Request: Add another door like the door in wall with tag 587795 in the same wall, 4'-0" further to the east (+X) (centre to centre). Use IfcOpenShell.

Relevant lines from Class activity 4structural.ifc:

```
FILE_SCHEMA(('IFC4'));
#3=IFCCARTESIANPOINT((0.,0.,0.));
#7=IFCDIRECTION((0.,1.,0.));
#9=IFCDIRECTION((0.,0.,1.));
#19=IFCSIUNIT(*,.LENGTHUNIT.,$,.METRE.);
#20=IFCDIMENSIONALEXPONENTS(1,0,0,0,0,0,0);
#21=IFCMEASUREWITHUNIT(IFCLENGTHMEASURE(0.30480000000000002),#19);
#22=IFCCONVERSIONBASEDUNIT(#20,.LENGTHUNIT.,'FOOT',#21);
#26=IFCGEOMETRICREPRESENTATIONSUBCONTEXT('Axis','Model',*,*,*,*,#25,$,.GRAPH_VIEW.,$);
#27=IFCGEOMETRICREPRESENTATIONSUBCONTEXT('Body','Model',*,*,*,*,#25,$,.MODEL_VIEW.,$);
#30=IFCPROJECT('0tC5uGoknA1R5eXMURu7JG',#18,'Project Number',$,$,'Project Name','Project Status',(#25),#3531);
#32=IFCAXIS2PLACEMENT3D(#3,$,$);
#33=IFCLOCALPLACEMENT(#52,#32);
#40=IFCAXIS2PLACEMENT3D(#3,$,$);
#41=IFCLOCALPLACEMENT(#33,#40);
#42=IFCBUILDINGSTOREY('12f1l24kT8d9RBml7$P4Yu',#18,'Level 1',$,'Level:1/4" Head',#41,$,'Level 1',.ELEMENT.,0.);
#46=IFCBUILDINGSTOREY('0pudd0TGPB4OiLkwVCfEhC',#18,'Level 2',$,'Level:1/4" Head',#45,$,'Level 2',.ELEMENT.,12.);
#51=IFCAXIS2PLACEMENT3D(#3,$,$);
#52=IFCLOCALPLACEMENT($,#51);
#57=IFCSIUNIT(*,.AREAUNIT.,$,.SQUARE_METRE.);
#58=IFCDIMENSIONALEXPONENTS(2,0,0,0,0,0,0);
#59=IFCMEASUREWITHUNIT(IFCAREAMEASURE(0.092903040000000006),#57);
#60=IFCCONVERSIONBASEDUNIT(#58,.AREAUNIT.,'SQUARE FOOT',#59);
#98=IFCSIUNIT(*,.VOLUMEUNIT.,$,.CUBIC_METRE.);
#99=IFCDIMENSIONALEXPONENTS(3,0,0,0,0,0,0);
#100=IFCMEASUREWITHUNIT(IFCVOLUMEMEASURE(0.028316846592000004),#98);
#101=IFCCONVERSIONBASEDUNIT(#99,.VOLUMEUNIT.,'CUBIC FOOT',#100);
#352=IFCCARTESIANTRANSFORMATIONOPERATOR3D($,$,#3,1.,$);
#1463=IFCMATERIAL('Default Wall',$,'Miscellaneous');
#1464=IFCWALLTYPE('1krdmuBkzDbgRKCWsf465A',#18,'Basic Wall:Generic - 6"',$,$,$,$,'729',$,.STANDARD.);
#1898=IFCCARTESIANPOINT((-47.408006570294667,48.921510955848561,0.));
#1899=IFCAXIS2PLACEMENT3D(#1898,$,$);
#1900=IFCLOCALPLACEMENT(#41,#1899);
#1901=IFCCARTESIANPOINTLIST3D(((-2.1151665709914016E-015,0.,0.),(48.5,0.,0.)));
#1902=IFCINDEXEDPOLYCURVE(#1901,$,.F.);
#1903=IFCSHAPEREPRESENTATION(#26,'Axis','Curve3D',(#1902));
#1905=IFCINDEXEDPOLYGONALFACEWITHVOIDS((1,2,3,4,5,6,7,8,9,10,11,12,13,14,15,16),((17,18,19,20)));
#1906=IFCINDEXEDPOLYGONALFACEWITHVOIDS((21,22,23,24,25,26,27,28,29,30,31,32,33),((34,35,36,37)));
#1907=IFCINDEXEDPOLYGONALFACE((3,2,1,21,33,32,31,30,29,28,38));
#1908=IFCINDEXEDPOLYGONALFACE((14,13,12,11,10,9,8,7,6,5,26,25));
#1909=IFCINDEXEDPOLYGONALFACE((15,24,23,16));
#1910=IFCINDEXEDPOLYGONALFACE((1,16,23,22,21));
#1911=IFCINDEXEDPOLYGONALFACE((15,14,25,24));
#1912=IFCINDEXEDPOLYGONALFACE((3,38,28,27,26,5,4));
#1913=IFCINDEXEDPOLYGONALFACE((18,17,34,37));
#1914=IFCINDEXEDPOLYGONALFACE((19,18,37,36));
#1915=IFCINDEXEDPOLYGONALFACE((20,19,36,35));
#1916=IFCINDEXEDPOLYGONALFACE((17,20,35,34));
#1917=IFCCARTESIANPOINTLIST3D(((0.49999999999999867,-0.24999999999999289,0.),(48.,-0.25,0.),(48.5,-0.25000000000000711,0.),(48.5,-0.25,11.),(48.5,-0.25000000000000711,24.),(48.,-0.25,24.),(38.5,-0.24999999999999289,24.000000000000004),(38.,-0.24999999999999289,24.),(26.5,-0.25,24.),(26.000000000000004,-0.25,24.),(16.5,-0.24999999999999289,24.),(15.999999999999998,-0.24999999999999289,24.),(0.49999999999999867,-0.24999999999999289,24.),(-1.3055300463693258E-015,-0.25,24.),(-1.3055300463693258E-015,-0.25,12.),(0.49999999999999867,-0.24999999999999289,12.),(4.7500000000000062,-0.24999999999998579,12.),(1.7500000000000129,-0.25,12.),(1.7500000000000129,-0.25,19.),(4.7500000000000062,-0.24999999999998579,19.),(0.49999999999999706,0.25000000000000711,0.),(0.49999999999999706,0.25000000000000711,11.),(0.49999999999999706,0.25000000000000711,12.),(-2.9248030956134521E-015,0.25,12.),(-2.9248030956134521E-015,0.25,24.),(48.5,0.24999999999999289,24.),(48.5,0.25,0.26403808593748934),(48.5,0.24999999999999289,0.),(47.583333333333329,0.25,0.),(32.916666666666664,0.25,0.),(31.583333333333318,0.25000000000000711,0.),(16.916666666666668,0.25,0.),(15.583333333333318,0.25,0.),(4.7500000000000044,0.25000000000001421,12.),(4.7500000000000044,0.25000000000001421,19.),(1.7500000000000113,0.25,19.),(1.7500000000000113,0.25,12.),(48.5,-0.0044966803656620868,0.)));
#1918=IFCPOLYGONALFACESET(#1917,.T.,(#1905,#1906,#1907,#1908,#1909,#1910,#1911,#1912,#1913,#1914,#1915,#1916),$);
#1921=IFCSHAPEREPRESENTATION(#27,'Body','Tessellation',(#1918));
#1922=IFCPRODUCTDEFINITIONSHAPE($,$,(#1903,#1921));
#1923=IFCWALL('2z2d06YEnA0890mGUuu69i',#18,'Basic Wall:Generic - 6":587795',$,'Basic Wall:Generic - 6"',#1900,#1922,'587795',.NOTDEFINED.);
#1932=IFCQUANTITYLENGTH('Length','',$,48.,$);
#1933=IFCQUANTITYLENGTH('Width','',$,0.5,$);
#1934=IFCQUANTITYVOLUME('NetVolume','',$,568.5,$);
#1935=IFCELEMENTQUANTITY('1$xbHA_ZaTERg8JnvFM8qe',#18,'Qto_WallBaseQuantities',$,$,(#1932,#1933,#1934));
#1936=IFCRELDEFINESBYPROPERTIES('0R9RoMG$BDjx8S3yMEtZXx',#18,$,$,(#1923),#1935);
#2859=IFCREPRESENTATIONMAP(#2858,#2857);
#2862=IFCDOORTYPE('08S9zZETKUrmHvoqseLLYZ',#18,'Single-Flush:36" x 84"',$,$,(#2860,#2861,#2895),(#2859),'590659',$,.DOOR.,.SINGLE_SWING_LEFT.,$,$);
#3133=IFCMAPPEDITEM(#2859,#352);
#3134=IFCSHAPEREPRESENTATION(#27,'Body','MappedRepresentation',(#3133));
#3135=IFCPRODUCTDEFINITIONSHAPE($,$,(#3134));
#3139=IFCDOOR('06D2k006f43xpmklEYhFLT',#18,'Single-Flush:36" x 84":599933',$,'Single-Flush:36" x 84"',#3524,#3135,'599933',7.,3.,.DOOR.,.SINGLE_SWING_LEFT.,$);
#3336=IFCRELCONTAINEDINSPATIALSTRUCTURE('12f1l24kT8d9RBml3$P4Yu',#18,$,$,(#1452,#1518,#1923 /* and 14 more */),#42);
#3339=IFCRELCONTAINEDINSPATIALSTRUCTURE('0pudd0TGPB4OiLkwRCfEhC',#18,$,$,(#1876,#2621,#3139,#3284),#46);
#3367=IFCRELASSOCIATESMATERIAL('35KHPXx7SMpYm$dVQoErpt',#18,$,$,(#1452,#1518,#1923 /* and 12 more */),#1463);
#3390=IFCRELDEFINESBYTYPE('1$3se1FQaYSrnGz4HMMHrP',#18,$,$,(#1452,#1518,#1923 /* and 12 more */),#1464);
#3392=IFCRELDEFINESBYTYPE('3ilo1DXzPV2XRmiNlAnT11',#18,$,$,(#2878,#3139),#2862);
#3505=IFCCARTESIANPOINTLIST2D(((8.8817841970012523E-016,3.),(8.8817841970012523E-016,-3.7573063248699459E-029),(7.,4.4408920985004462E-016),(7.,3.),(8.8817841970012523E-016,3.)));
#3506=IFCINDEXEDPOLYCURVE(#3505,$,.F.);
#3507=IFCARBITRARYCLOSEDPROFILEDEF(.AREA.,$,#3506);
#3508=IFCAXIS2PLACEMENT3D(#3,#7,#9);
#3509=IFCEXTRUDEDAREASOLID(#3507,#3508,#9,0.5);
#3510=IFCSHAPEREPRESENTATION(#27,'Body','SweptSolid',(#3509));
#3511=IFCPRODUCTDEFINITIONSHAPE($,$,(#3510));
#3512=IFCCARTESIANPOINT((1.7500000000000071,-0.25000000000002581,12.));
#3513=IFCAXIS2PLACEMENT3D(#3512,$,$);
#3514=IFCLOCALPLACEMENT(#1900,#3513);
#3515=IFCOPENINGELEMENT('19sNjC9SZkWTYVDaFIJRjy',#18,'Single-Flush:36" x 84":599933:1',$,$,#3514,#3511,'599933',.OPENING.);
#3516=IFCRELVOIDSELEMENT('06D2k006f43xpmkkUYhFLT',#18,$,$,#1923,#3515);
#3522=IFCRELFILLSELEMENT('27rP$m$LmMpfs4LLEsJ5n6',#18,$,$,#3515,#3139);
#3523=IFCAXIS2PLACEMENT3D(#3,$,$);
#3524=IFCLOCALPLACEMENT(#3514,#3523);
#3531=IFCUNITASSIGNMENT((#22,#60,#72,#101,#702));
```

```python
import ifcopenshell
import ifcopenshell.api.feature
import ifcopenshell.api.geometry
import ifcopenshell.api.pset
import ifcopenshell.api.root
import ifcopenshell.geom
import ifcopenshell.util.element
import ifcopenshell.util.placement
import ifcopenshell.util.shape
import ifcopenshell.util.unit

model = ifcopenshell.open("Class activity 4structural.ifc")
unit_scale = ifcopenshell.util.unit.calculate_unit_scale(model)
volume_scale = ifcopenshell.util.unit.calculate_unit_scale(model, "VOLUMEUNIT")
settings = ifcopenshell.geom.settings()


def volume(element):
    """Net volume in cubic metres, openings subtracted."""
    shape = ifcopenshell.geom.create_shape(settings, element)
    return ifcopenshell.util.shape.get_volume(shape.geometry)


def reuse_history(source, copy):
    """copy_class also copies each property set's owner history, people and application; keep the originals."""
    for rel in copy.IsDefinedBy:
        if rel.is_a("IfcRelDefinesByProperties") and (history := rel.RelatingPropertyDefinition.OwnerHistory):
            rel.RelatingPropertyDefinition.OwnerHistory = source.OwnerHistory
            ifcopenshell.util.element.remove_deep2(model, history)


door = model.by_guid("06D2k006f43xpmklEYhFLT")
opening = door.FillsVoids[0].RelatingOpeningElement
wall = opening.VoidsElements[0].RelatingBuildingElement
before = volume(wall)
shift = ifcopenshell.util.placement.get_local_placement(wall.ObjectPlacement)[:3, 0] * 48 * 0.0254 / unit_scale

# copy_class copies the void relationship, type, container and properties, but no geometry.
new_opening = ifcopenshell.api.root.copy_class(model, product=opening)
new_opening.Representation = ifcopenshell.util.element.copy_deep(
    model, opening.Representation, exclude=["IfcGeometricRepresentationContext", "IfcRepresentationMap"]
)
new_opening.Name = 'Single-Flush:36" x 84"'
new_opening.Tag = None
reuse_history(opening, new_opening)
new_door = ifcopenshell.api.root.copy_class(model, product=door)
new_door.Representation = ifcopenshell.util.element.copy_deep(
    model, door.Representation, exclude=["IfcGeometricRepresentationContext", "IfcRepresentationMap"]
)
new_door.Name = 'Single-Flush:36" x 84"'
new_door.Tag = None
reuse_history(door, new_door)
ifcopenshell.api.feature.add_filling(model, opening=new_opening, element=new_door)

for old, new in ((opening, new_opening), (door, new_door)):
    matrix = ifcopenshell.util.placement.get_local_placement(old.ObjectPlacement)
    matrix[:3, 3] += shift
    ifcopenshell.api.geometry.edit_object_placement(model, product=new, matrix=matrix, is_si=False)

after = volume(wall)

# Update the wall's stored quantities.
qto = model.by_id(ifcopenshell.util.element.get_pset(wall, "Qto_WallBaseQuantities", should_inherit=False)["id"])
ifcopenshell.api.pset.edit_qto(model, qto=qto, properties={"NetVolume": after / volume_scale})

print(f"wall volume {before:.3f} -> {after:.3f} m3")

model.write("Class activity 4structural_rev.ifc")
```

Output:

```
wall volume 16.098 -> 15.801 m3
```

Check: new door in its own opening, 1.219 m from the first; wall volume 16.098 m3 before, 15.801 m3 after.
